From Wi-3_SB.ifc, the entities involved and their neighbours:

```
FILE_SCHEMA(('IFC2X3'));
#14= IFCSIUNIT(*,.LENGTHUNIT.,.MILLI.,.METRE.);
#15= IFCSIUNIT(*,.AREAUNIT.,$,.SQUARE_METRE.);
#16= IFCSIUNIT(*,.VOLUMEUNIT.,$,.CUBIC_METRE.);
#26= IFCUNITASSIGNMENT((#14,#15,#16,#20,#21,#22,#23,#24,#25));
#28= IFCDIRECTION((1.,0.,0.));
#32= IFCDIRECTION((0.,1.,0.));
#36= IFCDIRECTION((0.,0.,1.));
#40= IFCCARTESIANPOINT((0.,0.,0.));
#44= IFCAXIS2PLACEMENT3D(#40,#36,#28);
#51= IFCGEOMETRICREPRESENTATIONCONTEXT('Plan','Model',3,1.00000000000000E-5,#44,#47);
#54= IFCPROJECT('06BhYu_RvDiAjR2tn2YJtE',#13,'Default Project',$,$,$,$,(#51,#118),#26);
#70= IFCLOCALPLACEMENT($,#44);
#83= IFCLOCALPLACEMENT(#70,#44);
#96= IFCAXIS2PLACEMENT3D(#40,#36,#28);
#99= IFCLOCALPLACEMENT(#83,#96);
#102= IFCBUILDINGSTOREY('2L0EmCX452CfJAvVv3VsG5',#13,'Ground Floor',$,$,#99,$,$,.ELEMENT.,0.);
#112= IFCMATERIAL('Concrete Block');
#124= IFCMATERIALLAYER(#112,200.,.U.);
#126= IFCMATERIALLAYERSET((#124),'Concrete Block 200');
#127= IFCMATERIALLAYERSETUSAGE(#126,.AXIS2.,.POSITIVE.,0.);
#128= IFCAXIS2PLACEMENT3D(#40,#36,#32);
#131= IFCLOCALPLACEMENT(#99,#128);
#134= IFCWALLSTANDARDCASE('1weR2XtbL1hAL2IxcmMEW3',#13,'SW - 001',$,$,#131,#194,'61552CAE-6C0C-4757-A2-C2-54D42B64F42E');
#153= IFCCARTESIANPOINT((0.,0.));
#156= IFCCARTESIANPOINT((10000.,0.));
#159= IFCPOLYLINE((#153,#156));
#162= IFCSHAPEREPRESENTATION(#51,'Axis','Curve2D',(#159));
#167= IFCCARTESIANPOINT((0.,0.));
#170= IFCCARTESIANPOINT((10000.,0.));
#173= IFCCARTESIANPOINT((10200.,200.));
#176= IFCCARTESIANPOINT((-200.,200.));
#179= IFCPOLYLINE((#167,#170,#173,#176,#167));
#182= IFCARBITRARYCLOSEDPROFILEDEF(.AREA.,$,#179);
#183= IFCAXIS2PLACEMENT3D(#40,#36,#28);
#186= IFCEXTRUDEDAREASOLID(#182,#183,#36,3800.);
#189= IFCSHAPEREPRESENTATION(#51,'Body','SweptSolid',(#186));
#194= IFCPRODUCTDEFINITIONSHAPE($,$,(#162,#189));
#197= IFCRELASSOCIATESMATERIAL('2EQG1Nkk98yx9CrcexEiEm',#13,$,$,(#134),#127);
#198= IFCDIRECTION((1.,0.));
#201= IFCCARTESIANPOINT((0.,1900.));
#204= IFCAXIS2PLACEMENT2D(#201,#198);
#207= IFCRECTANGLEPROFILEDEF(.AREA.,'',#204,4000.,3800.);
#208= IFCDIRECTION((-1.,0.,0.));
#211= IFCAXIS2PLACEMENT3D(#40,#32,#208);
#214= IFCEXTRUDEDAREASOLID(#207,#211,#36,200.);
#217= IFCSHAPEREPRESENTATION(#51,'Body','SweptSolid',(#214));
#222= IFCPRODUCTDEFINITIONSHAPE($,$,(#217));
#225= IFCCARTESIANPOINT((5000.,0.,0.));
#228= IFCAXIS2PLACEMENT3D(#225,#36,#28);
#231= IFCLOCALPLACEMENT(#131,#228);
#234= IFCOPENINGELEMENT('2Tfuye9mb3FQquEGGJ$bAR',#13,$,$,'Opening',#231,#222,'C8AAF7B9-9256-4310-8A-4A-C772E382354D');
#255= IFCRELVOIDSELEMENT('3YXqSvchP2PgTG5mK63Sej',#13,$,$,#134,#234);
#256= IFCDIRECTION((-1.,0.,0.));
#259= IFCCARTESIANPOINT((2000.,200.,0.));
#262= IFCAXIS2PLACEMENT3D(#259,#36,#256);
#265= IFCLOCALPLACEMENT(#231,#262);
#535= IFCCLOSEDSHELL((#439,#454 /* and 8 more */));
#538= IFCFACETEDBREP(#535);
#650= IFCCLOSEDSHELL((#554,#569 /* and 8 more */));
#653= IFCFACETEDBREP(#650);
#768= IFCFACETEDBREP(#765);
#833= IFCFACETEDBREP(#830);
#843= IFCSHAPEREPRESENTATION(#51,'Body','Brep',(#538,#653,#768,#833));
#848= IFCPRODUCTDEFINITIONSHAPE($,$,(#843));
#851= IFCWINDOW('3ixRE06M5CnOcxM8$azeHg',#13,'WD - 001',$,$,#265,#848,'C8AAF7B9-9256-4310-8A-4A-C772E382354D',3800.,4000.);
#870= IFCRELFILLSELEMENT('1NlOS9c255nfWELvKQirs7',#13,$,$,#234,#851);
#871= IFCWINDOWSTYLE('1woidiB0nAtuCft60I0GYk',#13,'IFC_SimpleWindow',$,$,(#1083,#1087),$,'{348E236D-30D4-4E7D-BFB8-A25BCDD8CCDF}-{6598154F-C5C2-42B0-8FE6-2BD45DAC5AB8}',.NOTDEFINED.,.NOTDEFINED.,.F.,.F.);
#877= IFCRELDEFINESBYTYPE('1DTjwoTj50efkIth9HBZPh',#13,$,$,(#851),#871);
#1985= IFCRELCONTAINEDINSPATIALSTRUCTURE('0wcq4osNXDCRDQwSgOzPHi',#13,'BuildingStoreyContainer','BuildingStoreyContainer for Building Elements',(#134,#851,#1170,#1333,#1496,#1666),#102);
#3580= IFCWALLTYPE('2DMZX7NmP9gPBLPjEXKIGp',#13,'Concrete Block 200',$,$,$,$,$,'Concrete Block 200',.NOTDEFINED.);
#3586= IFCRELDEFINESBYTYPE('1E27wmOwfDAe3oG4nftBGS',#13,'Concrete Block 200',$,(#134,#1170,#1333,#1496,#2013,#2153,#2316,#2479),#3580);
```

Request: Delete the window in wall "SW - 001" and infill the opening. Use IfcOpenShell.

```python
import ifcopenshell
import ifcopenshell.api.feature
import ifcopenshell.api.root
import ifcopenshell.geom
import ifcopenshell.util.shape

model = ifcopenshell.open("Wi-3_SB.ifc")
settings = ifcopenshell.geom.settings()


def volume(element):
    """Net volume in cubic metres, openings subtracted."""
    shape = ifcopenshell.geom.create_shape(settings, element)
    return ifcopenshell.util.shape.get_volume(shape.geometry)


window = model.by_guid("3ixRE06M5CnOcxM8$azeHg")
opening = window.FillsVoids[0].RelatingOpeningElement
wall = opening.VoidsElements[0].RelatingBuildingElement
before = volume(wall)

ifcopenshell.api.root.remove_product(model, product=window)
ifcopenshell.api.feature.remove_feature(model, feature=opening)

after = volume(wall)

print(f"wall volume {before:.3f} -> {after:.3f} m3")

model.write("Wi-3_SB-out.ifc")
```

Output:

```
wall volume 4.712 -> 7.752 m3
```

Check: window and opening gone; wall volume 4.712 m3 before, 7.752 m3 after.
